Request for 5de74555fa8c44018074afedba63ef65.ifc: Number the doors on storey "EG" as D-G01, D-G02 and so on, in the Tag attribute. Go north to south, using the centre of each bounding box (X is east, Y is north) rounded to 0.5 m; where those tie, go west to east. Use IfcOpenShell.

First a look at what the model holds.

```python
import ifcopenshell
import ifcopenshell.util.element
import ifcopenshell.util.placement

model = ifcopenshell.open("5de74555fa8c44018074afedba63ef65.ifc")
print(model.schema)
storey = next(s for s in model.by_type("IfcBuildingStorey") if s.Name == "EG")
doors = [e for e in ifcopenshell.util.element.get_decomposition(storey) if e.is_a("IfcDoor")]
for e in sorted(doors, key=lambda e: e.id()):
    origin = ifcopenshell.util.placement.get_local_placement(e.ObjectPlacement)[:3, 3]
    print(e.id(), e.Tag, e.Name, origin.round(2) + 0.0, sep=" | ")
```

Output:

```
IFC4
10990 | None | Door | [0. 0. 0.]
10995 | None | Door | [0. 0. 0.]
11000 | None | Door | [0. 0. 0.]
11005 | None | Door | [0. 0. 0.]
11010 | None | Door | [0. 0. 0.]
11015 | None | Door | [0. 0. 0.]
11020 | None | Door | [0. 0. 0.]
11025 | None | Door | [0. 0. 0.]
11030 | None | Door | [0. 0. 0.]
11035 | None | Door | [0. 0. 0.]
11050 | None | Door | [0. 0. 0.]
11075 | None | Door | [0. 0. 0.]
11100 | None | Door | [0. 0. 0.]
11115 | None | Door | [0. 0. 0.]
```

```python
import ifcopenshell
import ifcopenshell.geom
import ifcopenshell.util.element
import ifcopenshell.util.shape

model = ifcopenshell.open("5de74555fa8c44018074afedba63ef65.ifc")
settings = ifcopenshell.geom.settings()
settings.set("use-world-coords", True)


def centre(element):
    shape = ifcopenshell.geom.create_shape(settings, element)
    return ifcopenshell.util.shape.get_bbox_centroid(shape.geometry)


storey = next(s for s in model.by_type("IfcBuildingStorey") if s.Name == "EG")
doors = [e for e in ifcopenshell.util.element.get_decomposition(storey) if e.is_a("IfcDoor")]

# Insertion points can sit at a corner or the storey origin, so sort by the geometry (in metres).
centres = {e: centre(e) for e in doors}
doors.sort(key=lambda e: (-round(centres[e][1] / 0.5), centres[e][0]))

for i, e in enumerate(doors, start=1):
    number = f"D-G{i:02d}"
    e.Tag = number
    print(e.id(), number)

model.write("5de74555fa8c44018074afedba63ef65_rev.ifc")
```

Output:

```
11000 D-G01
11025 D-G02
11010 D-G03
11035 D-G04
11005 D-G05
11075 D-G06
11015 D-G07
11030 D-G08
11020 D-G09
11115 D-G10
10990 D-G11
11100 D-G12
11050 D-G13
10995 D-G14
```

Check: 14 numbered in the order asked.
